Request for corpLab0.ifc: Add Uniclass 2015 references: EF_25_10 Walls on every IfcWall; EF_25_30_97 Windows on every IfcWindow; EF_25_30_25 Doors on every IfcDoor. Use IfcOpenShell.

First a look at what the model holds.

```python
import ifcopenshell

model = ifcopenshell.open("corpLab0.ifc")
print(model.schema)
print("classifications:", [c.Name for c in model.by_type("IfcClassification")])
for ifc_class in ("IfcDoor", "IfcRoof", "IfcStair", "IfcWall", "IfcWindow"):
    print(ifc_class, len(model.by_type(ifc_class)))
```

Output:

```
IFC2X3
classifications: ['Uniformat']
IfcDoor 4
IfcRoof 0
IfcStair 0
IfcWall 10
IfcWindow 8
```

```python
import ifcopenshell
import ifcopenshell.api.classification

model = ifcopenshell.open("corpLab0.ifc")

# IFC2X3 requires Source and Edition and has no link from the project to the system.
system = model.create_entity("IfcClassification", Source="NBS", Edition="2015", Name="Uniclass 2015")

codes = {
    "IfcWall": ("EF_25_10", "Walls"),
    "IfcWindow": ("EF_25_30_97", "Windows"),
    "IfcDoor": ("EF_25_30_25", "Doors"),
}
for ifc_class, (code, name) in codes.items():
    products = model.by_type(ifc_class)
    ifcopenshell.api.classification.add_reference(
        model, products=products, classification=system, identification=code, name=name
    )
    print(code, len(products))

model.write("corpLab0_edited.ifc")
```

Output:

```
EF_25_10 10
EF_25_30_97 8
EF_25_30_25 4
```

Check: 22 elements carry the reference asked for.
